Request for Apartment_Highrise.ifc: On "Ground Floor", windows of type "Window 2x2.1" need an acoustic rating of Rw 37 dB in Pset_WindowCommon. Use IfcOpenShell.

First a look at what the model holds.

```python
import ifcopenshell
import ifcopenshell.util.element

model = ifcopenshell.open("Apartment_Highrise.ifc")
print(model.schema)
storey = next(s for s in model.by_type("IfcBuildingStorey") if s.Name == "Ground Floor")
windows = [e for e in ifcopenshell.util.element.get_decomposition(storey) if e.is_a("IfcWindow")]
seen = {}
for e in windows:
    element_type = ifcopenshell.util.element.get_type(e)
    key = (element_type.Name if element_type != e and element_type else None, ifcopenshell.util.element.get_pset(e, "Pset_WindowCommon", "AcousticRating"))
    seen[key] = seen.get(key, 0) + 1
for (name, value), count in sorted(seen.items(), key=str):
    print(count, "x", name, "|", value)
```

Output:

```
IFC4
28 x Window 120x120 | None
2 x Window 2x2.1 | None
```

```python
import ifcopenshell
import ifcopenshell.api.pset
import ifcopenshell.util.element

model = ifcopenshell.open("Apartment_Highrise.ifc")

storey = next(s for s in model.by_type("IfcBuildingStorey") if s.Name == "Ground Floor")
windows = [e for e in ifcopenshell.util.element.get_decomposition(storey) if e.is_a("IfcWindow")]

count = 0
for e in windows:
    element_type = ifcopenshell.util.element.get_type(e)
    if element_type in (None, e) or element_type.Name != "Window 2x2.1":
        continue
    found = ifcopenshell.util.element.get_pset(e, "Pset_WindowCommon", should_inherit=False)
    if found:
        pset = model.by_id(found["id"])
        if len(ifcopenshell.util.element.get_elements_by_pset(pset)) > 1:
            pset = ifcopenshell.api.pset.unshare_pset(model, products=[e], pset=pset)[0]
    else:
        pset = ifcopenshell.api.pset.add_pset(model, product=e, name="Pset_WindowCommon")
    ifcopenshell.api.pset.edit_pset(model, pset=pset, properties={"AcousticRating": "Rw 37 dB"})
    count += 1

print(count, "windows updated")

model.write("Apartment_Highrise_rev.ifc")
```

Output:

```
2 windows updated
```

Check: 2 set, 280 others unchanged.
